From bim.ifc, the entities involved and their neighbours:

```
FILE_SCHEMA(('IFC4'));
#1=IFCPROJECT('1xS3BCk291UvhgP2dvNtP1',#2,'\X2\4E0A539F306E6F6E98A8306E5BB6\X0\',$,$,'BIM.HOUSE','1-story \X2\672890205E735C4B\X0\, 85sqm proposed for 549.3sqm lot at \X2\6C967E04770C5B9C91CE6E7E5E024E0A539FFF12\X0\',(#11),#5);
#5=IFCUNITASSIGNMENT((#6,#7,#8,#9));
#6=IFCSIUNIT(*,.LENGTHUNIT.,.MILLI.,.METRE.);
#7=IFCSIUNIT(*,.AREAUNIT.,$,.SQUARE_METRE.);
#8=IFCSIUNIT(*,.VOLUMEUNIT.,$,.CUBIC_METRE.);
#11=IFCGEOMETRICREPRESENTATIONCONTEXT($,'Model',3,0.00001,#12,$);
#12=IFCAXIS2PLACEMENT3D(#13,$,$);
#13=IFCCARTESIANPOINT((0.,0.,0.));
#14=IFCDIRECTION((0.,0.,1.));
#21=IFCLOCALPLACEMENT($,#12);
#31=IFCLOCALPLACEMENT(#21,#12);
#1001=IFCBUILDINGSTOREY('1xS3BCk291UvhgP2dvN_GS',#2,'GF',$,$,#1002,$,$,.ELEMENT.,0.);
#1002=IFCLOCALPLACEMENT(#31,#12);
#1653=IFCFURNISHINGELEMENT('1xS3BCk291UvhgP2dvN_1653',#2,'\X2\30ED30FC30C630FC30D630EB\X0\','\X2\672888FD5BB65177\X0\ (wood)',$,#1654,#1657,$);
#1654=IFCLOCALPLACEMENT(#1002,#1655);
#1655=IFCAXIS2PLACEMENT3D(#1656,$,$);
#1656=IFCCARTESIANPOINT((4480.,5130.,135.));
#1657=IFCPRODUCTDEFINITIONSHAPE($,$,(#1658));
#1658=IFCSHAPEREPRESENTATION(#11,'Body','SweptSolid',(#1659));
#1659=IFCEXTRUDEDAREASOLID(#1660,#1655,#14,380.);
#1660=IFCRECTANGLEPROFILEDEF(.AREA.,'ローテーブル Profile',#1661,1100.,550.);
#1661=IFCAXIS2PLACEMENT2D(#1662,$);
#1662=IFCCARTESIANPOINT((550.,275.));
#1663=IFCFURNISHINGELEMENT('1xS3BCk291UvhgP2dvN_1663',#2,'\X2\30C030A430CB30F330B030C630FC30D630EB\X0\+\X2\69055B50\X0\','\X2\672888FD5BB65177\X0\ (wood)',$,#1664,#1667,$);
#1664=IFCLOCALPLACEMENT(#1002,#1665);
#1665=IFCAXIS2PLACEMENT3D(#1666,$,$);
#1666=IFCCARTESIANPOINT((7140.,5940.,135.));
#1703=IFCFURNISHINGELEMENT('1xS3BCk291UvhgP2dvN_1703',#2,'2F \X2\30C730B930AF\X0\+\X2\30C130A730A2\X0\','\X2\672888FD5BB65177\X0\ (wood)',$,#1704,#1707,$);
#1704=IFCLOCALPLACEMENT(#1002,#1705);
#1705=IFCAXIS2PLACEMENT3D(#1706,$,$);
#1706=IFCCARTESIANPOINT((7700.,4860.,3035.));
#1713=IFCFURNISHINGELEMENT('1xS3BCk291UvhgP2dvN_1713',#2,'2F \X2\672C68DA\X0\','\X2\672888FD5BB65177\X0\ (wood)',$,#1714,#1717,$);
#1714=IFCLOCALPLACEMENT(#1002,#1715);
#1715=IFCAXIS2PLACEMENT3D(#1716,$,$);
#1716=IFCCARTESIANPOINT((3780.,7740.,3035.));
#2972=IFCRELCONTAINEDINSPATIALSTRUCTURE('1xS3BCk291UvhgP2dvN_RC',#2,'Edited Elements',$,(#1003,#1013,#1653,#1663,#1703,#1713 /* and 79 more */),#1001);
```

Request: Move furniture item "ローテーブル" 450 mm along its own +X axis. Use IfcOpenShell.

```python
import ifcopenshell
import ifcopenshell.api.geometry
import ifcopenshell.util.placement
import ifcopenshell.util.unit

model = ifcopenshell.open("bim.ifc")
unit_scale = ifcopenshell.util.unit.calculate_unit_scale(model)

item = model.by_guid("1xS3BCk291UvhgP2dvN_1653")
matrix = ifcopenshell.util.placement.get_local_placement(item.ObjectPlacement)
matrix[:3, 3] += matrix[:3, 0] * 0.45 / unit_scale
ifcopenshell.api.geometry.edit_object_placement(model, product=item, matrix=matrix, is_si=False)

print(ifcopenshell.util.placement.get_local_placement(item.ObjectPlacement).round(3) + 0.0)

model.write("bim_updated.ifc")
```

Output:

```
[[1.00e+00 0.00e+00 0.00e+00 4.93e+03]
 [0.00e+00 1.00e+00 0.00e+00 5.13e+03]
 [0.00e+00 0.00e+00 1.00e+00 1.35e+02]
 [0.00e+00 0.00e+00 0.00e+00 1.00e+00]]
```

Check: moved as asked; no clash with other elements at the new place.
